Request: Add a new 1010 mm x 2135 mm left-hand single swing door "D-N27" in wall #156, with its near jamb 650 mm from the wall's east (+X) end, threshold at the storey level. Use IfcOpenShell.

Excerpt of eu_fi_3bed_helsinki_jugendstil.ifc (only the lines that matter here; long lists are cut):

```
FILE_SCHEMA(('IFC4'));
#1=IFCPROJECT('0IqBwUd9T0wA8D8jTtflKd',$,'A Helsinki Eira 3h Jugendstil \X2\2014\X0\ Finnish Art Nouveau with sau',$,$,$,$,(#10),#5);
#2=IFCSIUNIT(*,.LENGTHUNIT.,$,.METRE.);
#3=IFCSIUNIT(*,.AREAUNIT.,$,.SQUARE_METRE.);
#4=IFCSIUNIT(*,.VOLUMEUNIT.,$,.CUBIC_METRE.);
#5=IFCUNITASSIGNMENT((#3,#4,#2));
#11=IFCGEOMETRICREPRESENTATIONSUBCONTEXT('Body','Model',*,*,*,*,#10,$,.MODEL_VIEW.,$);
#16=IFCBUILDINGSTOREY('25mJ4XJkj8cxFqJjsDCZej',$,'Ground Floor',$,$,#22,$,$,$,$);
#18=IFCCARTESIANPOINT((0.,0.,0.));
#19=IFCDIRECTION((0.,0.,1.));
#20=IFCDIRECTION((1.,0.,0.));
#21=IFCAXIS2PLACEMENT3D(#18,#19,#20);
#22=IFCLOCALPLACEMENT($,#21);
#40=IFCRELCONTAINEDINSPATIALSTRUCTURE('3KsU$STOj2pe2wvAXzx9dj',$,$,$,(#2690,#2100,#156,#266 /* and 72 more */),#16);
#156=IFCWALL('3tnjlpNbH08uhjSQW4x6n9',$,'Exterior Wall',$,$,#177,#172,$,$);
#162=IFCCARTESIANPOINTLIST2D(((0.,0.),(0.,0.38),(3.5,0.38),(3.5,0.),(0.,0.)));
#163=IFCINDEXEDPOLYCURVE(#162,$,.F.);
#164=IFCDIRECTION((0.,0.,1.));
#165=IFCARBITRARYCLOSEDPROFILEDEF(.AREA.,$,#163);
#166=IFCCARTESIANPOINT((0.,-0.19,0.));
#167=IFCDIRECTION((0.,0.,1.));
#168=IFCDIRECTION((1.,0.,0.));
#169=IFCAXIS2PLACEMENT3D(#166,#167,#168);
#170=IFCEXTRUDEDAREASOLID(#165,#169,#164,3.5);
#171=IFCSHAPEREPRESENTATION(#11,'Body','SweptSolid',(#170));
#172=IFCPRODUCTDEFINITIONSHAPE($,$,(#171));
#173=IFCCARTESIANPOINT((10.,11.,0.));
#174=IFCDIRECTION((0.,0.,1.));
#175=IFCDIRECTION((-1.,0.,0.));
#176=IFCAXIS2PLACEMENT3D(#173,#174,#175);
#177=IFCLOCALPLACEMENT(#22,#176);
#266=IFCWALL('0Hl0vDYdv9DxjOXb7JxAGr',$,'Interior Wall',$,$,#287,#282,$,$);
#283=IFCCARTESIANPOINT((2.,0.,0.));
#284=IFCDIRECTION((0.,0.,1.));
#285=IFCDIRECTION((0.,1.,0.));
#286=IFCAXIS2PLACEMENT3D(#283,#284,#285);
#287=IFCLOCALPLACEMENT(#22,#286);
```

```python
import numpy as np
import ifcopenshell
import ifcopenshell.api.feature
import ifcopenshell.api.geometry
import ifcopenshell.api.root
import ifcopenshell.api.spatial
import ifcopenshell.geom
import ifcopenshell.util.element
import ifcopenshell.util.placement
import ifcopenshell.util.representation
import ifcopenshell.util.shape
import ifcopenshell.util.unit

model = ifcopenshell.open("eu_fi_3bed_helsinki_jugendstil.ifc")
unit_scale = ifcopenshell.util.unit.calculate_unit_scale(model)
settings = ifcopenshell.geom.settings()


def volume(element):
    """Net volume in cubic metres, openings subtracted."""
    shape = ifcopenshell.geom.create_shape(settings, element)
    return ifcopenshell.util.shape.get_volume(shape.geometry)


wall = model.by_id(156)
storey = ifcopenshell.util.element.get_container(wall, ifc_class="IfcBuildingStorey")
context = ifcopenshell.util.representation.get_context(model, "Model", "Body", "MODEL_VIEW")
before = volume(wall)

width, height, from_end, sill = 1.01, 2.135, 0.65, 0.0  # metres

# The wall runs along its own X axis, and the end named is its -X end.
wall_shape = ifcopenshell.geom.create_shape(settings, wall)
x, y, z = ifcopenshell.util.shape.get_vertices(wall_shape.geometry).T
start = x.min() + from_end
face, thickness = float(y.min()), float(y.max() - y.min())
wall_matrix = ifcopenshell.util.placement.get_local_placement(wall.ObjectPlacement)
level = ifcopenshell.util.placement.get_local_placement(storey.ObjectPlacement)[2, 3]


def in_wall(x, y):
    """Placement at x, y metres in the wall's axes, at sill height."""
    matrix = wall_matrix.copy()
    matrix[:, 3] = wall_matrix @ np.array([x / unit_scale, y / unit_scale, 0.0, 1.0])
    matrix[2, 3] = level + sill / unit_scale
    return matrix


# Opening: a box that overshoots both wall faces by 50 mm.
opening = ifcopenshell.api.root.create_entity(model, ifc_class="IfcOpeningElement", predefined_type="OPENING")
box = ifcopenshell.api.geometry.add_wall_representation(
    model, context=context, length=width, height=height, thickness=thickness + 0.1
)
ifcopenshell.api.geometry.assign_representation(model, product=opening, representation=box)
ifcopenshell.api.geometry.edit_object_placement(model, product=opening, matrix=in_wall(start, face - 0.05), is_si=False)
ifcopenshell.api.feature.add_feature(model, feature=opening, element=wall)

door = ifcopenshell.api.root.create_entity(model, ifc_class="IfcDoor", name="D-N27", predefined_type="DOOR")
door.OverallWidth, door.OverallHeight = width / unit_scale, height / unit_scale
door.OperationType = "SINGLE_SWING_LEFT"
body = ifcopenshell.api.geometry.add_door_representation(
    model,
    context=context,
    overall_width=door.OverallWidth,
    overall_height=door.OverallHeight,
    operation_type="SINGLE_SWING_LEFT",
    lining_properties={"LiningDepth": thickness / unit_scale, "ThresholdDepth": thickness / unit_scale},
)
ifcopenshell.api.geometry.assign_representation(model, product=door, representation=body)
ifcopenshell.api.spatial.assign_container(model, products=[door], relating_structure=storey)
ifcopenshell.api.feature.add_filling(model, opening=opening, element=door)

# The lining spans the wall, so the door starts at the wall face.
ifcopenshell.api.geometry.edit_object_placement(model, product=door, matrix=in_wall(start, face), is_si=False)

after = volume(wall)

print(f"wall volume {before:.3f} -> {after:.3f} m3")

model.write("eu_fi_3bed_helsinki_jugendstil_updated.ifc")
```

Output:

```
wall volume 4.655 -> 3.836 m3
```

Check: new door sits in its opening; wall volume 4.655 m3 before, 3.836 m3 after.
